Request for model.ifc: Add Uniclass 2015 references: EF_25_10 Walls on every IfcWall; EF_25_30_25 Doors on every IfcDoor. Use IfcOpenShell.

First a look at what the model holds.

```python
import ifcopenshell

model = ifcopenshell.open("model.ifc")
print(model.schema)
print("classifications:", [c.Name for c in model.by_type("IfcClassification")])
for ifc_class in ("IfcDoor", "IfcRoof", "IfcStair", "IfcWall", "IfcWindow"):
    print(ifc_class, len(model.by_type(ifc_class)))
```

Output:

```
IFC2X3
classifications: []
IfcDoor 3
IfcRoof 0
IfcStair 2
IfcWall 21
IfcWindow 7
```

```python
import ifcopenshell
import ifcopenshell.api.classification

model = ifcopenshell.open("model.ifc")

# IFC2X3 requires Source and Edition and has no link from the project to the system.
system = model.create_entity("IfcClassification", Source="NBS", Edition="2015", Name="Uniclass 2015")

codes = {
    "IfcWall": ("EF_25_10", "Walls"),
    "IfcDoor": ("EF_25_30_25", "Doors"),
}
for ifc_class, (code, name) in codes.items():
    products = model.by_type(ifc_class)
    ifcopenshell.api.classification.add_reference(
        model, products=products, classification=system, identification=code, name=name
    )
    print(code, len(products))

model.write("model_updated.ifc")
```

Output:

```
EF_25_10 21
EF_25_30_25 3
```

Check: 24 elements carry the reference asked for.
